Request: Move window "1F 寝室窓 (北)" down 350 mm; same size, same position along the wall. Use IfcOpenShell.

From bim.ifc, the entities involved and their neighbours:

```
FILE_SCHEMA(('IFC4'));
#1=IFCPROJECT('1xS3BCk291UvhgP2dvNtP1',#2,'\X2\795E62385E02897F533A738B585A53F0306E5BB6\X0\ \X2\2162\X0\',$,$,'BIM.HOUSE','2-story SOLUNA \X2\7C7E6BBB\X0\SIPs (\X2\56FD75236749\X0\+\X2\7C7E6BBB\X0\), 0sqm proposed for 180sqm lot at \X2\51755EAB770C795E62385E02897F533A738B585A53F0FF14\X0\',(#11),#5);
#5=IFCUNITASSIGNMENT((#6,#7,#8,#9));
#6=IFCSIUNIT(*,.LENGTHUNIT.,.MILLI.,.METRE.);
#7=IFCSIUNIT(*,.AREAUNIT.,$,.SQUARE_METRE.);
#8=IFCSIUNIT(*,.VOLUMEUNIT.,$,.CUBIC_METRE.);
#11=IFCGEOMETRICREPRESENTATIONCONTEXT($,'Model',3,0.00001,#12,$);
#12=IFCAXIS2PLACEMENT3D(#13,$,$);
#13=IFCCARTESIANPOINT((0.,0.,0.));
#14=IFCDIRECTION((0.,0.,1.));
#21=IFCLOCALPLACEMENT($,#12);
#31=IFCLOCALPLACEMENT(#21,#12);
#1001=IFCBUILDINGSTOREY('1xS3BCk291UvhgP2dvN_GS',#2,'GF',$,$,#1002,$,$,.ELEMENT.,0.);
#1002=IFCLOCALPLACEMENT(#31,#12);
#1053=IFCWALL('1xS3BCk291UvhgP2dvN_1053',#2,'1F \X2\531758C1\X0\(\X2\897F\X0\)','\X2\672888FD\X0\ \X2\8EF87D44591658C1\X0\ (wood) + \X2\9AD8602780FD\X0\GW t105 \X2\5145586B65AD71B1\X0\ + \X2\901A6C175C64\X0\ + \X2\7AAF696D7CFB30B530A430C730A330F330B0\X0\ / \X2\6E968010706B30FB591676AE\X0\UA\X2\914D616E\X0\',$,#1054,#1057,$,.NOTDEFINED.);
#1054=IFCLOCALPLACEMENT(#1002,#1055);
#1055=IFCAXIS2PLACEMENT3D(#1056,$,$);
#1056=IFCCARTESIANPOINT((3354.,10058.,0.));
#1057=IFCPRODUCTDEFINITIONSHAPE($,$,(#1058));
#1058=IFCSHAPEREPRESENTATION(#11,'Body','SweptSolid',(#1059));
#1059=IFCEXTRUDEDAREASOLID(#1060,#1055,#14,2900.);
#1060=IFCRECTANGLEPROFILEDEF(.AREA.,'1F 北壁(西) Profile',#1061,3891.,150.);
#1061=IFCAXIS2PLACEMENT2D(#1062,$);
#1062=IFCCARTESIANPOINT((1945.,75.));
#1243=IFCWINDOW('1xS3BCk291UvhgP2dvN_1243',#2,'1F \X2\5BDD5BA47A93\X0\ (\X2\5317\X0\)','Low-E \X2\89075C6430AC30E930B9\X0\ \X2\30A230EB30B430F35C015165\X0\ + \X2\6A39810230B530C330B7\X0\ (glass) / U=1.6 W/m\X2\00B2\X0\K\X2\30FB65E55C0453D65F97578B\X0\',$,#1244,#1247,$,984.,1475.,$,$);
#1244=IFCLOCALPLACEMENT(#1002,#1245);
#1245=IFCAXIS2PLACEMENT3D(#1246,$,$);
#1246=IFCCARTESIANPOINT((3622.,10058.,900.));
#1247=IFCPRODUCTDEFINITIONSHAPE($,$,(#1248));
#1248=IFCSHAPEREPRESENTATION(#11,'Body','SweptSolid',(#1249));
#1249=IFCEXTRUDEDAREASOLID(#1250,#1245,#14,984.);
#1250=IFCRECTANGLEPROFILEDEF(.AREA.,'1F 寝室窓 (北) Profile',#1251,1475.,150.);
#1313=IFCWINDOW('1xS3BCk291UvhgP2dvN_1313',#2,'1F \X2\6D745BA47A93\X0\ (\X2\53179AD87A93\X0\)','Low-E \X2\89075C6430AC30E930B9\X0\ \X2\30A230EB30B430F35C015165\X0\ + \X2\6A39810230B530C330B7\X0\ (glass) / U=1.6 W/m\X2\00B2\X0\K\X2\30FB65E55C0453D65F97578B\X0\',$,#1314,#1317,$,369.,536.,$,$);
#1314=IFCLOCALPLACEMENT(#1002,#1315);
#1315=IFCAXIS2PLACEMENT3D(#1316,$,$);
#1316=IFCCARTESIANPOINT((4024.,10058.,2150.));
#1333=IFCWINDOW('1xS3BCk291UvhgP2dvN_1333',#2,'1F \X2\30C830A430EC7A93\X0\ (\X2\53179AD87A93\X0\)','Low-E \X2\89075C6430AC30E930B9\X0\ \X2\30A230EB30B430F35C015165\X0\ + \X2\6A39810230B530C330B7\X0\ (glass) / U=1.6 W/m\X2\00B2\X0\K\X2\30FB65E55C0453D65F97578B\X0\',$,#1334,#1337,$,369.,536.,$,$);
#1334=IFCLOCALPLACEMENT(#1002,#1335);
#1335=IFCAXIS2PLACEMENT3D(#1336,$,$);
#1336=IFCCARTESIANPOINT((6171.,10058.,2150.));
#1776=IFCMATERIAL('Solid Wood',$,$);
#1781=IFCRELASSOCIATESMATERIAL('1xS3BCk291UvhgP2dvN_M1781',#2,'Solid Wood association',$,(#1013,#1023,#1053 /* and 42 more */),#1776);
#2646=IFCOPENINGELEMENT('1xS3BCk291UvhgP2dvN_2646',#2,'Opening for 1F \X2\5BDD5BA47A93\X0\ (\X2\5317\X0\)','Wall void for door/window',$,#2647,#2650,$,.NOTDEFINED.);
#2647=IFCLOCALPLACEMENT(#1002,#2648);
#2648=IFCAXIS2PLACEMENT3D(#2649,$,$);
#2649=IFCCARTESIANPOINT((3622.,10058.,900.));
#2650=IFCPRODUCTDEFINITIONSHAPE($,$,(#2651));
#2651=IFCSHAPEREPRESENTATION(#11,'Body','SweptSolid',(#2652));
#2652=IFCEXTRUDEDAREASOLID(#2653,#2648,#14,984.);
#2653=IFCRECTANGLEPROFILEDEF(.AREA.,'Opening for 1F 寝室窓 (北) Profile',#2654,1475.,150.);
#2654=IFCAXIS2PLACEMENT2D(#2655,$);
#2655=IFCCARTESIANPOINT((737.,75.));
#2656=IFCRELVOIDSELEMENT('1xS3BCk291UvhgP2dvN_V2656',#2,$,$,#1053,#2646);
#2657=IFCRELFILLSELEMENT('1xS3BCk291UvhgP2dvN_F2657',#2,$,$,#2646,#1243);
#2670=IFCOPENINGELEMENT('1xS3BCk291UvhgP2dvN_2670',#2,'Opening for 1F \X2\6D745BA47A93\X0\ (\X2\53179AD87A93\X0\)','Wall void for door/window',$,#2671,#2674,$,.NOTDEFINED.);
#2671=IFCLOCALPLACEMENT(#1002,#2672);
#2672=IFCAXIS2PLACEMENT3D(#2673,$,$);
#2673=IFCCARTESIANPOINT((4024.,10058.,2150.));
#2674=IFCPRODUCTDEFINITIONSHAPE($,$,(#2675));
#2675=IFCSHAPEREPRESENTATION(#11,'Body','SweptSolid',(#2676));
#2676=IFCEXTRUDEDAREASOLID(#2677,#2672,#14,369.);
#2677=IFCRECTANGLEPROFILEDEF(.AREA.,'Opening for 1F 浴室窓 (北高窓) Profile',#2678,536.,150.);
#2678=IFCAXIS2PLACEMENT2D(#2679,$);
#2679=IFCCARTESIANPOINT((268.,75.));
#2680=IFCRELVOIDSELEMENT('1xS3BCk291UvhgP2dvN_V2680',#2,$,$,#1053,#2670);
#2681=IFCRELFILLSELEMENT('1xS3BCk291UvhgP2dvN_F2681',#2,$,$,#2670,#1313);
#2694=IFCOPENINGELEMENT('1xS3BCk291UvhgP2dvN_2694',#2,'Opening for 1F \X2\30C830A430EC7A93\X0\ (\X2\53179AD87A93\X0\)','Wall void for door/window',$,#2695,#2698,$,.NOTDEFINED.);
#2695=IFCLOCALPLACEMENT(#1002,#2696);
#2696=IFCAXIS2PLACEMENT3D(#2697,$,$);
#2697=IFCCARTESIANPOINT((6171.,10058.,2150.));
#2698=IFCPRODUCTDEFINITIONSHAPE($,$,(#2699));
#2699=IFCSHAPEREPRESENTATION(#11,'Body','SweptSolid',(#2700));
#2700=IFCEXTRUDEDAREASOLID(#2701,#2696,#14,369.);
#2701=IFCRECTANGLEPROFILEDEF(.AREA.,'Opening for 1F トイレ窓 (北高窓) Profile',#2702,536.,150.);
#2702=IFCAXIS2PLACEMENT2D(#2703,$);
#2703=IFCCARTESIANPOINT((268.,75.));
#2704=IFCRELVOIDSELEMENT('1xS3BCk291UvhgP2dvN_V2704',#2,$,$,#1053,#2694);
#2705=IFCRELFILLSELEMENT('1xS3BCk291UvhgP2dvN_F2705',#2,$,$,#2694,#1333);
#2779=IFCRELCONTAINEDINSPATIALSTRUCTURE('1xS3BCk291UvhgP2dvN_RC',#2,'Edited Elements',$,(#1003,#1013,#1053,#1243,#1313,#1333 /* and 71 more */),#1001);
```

```python
import numpy as np
import ifcopenshell
import ifcopenshell.api.geometry
import ifcopenshell.util.placement
import ifcopenshell.util.unit

model = ifcopenshell.open("bim.ifc")
unit_scale = ifcopenshell.util.unit.calculate_unit_scale(model)

window = model.by_id(1243)
opening = window.FillsVoids[0].RelatingOpeningElement
dz = -350.0

shift = np.array([0.0, 0.0, dz])
# The window is not placed relative to its opening, so move both.
for product in (opening, window):
    matrix = ifcopenshell.util.placement.get_local_placement(product.ObjectPlacement)
    matrix[:3, 3] += shift
    ifcopenshell.api.geometry.edit_object_placement(model, product=product, matrix=matrix, is_si=False)

print(f"moved by {dz * unit_scale:+.3f} m")

model.write("bim_rev.ifc")
```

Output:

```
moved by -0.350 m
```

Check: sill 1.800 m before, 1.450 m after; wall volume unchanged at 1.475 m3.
